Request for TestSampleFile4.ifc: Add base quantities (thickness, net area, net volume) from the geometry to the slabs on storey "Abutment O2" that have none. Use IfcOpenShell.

First a look at what the model holds.

```python
import ifcopenshell
import ifcopenshell.util.element
import ifcopenshell.util.unit

model = ifcopenshell.open("TestSampleFile4.ifc")
print(model.schema)
for unit_type in ("LENGTHUNIT", "AREAUNIT", "VOLUMEUNIT"):
    print(unit_type, ifcopenshell.util.unit.calculate_unit_scale(model, unit_type))
storey = next(s for s in model.by_type("IfcBuildingStorey") if s.Name == "Abutment O2")
slabs = [e for e in ifcopenshell.util.element.get_decomposition(storey) if e.is_a("IfcSlab")]
for e in sorted(slabs, key=lambda e: e.id()):
    print(e.id(), e.is_a(), e.Name, list(ifcopenshell.util.element.get_psets(e, qtos_only=True)), sep=" | ")
```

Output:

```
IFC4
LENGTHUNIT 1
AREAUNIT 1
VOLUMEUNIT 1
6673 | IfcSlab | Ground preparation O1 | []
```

```python
import ifcopenshell
import ifcopenshell.api.pset
import ifcopenshell.geom
import ifcopenshell.util.element
import ifcopenshell.util.shape
import ifcopenshell.util.unit

model = ifcopenshell.open("TestSampleFile4.ifc")
unit_scale = ifcopenshell.util.unit.calculate_unit_scale(model)
area_scale = ifcopenshell.util.unit.calculate_unit_scale(model, "AREAUNIT")
volume_scale = ifcopenshell.util.unit.calculate_unit_scale(model, "VOLUMEUNIT")
settings = ifcopenshell.geom.settings()

storey = next(s for s in model.by_type("IfcBuildingStorey") if s.Name == "Abutment O2")
slabs = [e for e in ifcopenshell.util.element.get_decomposition(storey) if e.is_a("IfcSlab")]

for e in sorted(slabs, key=lambda e: e.id()):
    if ifcopenshell.util.element.get_psets(e, qtos_only=True, should_inherit=False):
        continue
    # Geometry comes back in metres, in the element's own axes.
    shape = ifcopenshell.geom.create_shape(settings, e)
    values = {
        "Width": ifcopenshell.util.shape.get_z(shape.geometry) / unit_scale,
        "NetArea": ifcopenshell.util.shape.get_footprint_area(shape.geometry) / area_scale,
        "NetVolume": ifcopenshell.util.shape.get_volume(shape.geometry) / volume_scale,
    }
    qto = ifcopenshell.api.pset.add_qto(model, product=e, name="Qto_SlabBaseQuantities")
    ifcopenshell.api.pset.edit_qto(model, qto=qto, properties=values)
    print(e.id(), {k: round(v, 3) for k, v in values.items()})

model.write("TestSampleFile4-out.ifc")
```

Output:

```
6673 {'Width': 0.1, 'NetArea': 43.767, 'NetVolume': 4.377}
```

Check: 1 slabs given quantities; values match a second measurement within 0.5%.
